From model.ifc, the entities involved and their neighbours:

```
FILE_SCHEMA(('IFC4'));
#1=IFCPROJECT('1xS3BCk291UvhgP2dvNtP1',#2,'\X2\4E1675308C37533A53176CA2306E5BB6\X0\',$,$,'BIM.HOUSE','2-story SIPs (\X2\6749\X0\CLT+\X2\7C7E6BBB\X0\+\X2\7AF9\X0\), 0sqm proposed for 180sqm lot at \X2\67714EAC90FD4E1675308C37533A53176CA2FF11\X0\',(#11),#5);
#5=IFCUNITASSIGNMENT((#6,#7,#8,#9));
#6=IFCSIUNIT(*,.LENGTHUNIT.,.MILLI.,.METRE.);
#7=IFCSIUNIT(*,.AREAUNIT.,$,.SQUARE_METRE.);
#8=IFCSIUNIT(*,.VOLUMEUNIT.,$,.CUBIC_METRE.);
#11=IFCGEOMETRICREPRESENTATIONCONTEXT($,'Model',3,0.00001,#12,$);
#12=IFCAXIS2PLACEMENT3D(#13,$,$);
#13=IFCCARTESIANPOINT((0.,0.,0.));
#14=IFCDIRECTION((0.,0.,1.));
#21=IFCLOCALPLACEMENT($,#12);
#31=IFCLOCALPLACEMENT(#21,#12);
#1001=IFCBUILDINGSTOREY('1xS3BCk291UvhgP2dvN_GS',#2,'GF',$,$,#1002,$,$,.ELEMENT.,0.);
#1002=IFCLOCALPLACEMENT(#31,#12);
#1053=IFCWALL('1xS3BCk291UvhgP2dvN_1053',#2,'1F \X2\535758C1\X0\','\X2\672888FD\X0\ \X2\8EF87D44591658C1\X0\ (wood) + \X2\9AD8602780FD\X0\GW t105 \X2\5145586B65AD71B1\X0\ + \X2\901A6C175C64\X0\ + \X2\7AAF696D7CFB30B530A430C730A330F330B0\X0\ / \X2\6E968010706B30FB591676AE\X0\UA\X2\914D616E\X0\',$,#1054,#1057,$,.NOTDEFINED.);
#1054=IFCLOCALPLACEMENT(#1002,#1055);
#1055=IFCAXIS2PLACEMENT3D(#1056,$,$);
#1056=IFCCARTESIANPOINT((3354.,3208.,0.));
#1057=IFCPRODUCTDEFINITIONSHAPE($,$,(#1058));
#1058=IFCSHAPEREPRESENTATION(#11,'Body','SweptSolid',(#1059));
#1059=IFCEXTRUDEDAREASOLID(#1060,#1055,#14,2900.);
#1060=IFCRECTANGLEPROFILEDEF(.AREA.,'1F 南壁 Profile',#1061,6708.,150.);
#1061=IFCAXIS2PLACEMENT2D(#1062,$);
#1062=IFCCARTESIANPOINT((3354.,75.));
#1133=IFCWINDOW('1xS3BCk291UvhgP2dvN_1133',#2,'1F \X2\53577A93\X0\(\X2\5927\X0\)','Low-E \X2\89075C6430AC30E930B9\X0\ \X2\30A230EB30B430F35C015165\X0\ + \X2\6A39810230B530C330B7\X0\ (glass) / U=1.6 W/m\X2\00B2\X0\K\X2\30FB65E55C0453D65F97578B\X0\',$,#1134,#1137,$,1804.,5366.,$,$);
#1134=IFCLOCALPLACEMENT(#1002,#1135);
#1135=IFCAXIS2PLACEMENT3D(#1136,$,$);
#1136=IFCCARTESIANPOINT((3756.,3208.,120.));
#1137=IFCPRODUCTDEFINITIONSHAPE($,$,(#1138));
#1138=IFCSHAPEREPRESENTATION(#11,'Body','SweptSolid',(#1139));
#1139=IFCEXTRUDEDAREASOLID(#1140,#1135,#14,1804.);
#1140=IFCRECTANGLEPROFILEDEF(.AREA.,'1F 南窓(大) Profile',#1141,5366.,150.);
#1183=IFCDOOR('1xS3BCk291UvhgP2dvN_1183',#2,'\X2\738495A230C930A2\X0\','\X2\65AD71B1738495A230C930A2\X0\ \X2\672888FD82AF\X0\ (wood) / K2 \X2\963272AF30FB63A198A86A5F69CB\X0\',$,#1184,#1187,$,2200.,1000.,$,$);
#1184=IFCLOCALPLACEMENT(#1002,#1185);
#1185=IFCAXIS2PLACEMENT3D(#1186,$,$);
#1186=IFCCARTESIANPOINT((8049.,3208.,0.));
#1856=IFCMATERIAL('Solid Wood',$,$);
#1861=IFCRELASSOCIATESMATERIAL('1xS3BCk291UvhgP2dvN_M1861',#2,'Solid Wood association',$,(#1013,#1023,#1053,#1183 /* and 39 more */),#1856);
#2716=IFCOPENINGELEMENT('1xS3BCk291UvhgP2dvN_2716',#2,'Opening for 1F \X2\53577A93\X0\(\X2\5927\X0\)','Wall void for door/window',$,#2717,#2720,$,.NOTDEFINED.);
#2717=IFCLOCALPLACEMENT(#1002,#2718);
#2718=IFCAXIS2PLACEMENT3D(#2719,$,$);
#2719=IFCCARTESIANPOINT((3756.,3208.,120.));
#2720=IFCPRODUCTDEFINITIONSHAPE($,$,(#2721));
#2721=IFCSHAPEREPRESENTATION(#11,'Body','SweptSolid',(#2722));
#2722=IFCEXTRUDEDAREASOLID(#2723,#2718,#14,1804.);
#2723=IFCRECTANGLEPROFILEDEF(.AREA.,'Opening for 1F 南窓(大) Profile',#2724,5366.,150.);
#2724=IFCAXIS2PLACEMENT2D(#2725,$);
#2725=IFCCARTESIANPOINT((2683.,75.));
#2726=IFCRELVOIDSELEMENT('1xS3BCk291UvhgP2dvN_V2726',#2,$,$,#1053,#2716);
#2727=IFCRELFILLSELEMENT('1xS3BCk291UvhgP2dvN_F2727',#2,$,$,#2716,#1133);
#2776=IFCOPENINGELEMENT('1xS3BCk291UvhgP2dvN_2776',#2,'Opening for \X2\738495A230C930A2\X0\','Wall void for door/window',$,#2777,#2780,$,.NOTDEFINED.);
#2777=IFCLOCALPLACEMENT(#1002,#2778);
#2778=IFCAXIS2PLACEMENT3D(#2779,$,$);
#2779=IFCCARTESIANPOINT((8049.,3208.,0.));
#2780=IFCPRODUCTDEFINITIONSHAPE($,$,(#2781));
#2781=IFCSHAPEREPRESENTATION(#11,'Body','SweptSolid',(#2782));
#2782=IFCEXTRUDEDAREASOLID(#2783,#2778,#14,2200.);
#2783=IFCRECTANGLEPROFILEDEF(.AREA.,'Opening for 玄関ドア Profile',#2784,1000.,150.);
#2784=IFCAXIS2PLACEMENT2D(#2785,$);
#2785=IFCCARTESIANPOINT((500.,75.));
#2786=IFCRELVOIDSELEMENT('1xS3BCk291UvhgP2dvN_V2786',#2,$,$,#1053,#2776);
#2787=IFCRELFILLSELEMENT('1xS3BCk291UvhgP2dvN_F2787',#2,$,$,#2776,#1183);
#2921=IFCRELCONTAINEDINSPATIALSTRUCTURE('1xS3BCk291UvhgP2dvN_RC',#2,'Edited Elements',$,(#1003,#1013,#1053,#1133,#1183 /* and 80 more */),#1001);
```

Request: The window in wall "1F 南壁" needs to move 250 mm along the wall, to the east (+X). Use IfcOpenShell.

```python
import ifcopenshell
import ifcopenshell.api.geometry
import ifcopenshell.util.placement
import ifcopenshell.util.unit

model = ifcopenshell.open("model.ifc")
unit_scale = ifcopenshell.util.unit.calculate_unit_scale(model)

window = model.by_guid("1xS3BCk291UvhgP2dvN_1133")
opening = window.FillsVoids[0].RelatingOpeningElement
wall = opening.VoidsElements[0].RelatingBuildingElement

wall_matrix = ifcopenshell.util.placement.get_local_placement(wall.ObjectPlacement)
shift = wall_matrix[:3, 0] * 0.25 / unit_scale
before = ifcopenshell.util.placement.get_local_placement(window.ObjectPlacement)[:3, 3].copy()

# The window is not placed relative to its opening, so move both.
for product in (opening, window):
    matrix = ifcopenshell.util.placement.get_local_placement(product.ObjectPlacement)
    matrix[:3, 3] += shift
    ifcopenshell.api.geometry.edit_object_placement(model, product=product, matrix=matrix, is_si=False)

after = ifcopenshell.util.placement.get_local_placement(window.ObjectPlacement)[:3, 3]
print("window moved by", (after - before).round(3) + 0.0)

model.write("model_v2.ifc")
```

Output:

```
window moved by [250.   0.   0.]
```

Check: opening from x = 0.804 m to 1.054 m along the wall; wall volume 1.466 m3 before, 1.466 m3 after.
